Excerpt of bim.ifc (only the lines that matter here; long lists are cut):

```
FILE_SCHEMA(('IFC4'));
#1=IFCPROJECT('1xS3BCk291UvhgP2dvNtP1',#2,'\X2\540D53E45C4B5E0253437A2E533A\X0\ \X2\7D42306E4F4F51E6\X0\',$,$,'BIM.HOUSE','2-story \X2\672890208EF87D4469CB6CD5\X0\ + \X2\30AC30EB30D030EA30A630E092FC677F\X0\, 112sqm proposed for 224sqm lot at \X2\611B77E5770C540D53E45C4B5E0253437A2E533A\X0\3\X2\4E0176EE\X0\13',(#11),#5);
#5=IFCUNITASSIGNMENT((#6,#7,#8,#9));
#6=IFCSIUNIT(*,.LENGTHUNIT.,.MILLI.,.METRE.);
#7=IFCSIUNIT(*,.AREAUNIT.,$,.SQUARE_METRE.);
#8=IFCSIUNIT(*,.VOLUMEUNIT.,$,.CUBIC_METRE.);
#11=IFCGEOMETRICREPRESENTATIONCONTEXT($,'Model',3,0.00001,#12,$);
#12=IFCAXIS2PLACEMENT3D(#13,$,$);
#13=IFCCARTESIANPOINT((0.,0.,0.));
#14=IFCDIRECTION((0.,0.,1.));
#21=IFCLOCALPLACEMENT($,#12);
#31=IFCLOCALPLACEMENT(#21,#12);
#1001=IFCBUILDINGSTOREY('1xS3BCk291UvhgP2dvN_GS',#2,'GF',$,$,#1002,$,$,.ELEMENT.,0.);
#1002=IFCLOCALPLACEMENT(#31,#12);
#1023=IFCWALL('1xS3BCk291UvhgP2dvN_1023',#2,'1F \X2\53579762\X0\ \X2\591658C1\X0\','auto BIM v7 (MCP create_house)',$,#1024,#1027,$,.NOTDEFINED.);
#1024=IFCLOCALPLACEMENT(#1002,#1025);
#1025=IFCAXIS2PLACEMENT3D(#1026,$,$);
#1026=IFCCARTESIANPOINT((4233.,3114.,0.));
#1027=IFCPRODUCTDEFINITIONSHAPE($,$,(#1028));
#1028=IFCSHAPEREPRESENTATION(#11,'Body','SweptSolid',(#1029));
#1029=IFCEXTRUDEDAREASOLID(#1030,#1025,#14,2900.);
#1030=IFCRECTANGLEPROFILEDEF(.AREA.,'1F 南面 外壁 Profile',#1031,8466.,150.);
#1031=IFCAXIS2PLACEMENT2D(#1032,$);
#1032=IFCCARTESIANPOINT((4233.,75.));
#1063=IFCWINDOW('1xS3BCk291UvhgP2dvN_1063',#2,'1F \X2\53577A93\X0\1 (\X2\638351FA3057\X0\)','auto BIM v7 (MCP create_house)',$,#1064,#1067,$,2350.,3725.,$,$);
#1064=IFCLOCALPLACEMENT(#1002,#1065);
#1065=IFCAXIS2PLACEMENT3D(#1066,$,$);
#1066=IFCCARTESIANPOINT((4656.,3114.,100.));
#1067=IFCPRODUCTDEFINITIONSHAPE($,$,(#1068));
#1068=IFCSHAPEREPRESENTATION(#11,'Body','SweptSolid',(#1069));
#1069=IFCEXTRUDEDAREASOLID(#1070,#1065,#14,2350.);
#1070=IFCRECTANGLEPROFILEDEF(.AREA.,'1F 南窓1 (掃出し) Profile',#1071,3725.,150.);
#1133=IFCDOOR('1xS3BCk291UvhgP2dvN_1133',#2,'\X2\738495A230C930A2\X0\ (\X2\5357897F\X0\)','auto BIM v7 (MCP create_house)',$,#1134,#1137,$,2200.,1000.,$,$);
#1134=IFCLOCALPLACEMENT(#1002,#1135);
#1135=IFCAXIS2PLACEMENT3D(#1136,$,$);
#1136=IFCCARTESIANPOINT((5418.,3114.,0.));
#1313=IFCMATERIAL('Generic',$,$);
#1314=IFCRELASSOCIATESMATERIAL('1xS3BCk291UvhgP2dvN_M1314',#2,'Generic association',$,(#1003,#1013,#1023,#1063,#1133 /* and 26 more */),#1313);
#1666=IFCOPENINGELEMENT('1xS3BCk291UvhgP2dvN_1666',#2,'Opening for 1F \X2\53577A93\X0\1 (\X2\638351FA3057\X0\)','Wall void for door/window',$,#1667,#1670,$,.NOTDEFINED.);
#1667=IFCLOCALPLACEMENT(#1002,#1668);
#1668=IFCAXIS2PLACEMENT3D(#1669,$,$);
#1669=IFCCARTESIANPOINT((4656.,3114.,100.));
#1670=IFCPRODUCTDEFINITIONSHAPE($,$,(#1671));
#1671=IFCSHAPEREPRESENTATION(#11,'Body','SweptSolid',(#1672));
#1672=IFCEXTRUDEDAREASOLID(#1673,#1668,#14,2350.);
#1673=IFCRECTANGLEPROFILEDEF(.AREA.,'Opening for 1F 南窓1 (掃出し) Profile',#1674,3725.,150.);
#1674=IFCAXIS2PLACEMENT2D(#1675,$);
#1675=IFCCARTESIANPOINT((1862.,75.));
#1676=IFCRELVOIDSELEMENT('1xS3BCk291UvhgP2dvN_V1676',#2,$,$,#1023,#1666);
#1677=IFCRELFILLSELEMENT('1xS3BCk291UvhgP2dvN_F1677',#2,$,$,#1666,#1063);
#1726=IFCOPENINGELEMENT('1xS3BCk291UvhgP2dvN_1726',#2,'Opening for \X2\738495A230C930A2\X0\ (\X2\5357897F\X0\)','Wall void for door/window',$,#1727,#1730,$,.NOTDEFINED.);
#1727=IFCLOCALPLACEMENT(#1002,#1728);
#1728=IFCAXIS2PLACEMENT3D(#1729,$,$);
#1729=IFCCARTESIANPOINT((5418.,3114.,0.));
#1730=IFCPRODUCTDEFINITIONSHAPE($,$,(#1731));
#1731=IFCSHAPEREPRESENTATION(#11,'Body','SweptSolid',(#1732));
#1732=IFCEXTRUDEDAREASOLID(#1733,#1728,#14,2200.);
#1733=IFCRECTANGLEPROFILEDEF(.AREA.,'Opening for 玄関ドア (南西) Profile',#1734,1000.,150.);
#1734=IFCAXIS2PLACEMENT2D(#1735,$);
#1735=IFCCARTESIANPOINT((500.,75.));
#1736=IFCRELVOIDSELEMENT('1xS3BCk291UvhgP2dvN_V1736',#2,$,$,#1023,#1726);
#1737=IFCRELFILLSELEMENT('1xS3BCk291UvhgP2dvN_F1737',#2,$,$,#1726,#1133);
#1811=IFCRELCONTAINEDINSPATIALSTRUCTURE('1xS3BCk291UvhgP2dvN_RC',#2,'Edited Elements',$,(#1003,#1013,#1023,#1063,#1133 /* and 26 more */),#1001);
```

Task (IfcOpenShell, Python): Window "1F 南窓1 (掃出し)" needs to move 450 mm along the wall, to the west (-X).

```python
import ifcopenshell
import ifcopenshell.api.geometry
import ifcopenshell.util.placement
import ifcopenshell.util.unit

model = ifcopenshell.open("bim.ifc")
unit_scale = ifcopenshell.util.unit.calculate_unit_scale(model)

window = model.by_guid("1xS3BCk291UvhgP2dvN_1063")
opening = window.FillsVoids[0].RelatingOpeningElement
wall = opening.VoidsElements[0].RelatingBuildingElement

wall_matrix = ifcopenshell.util.placement.get_local_placement(wall.ObjectPlacement)
shift = wall_matrix[:3, 0] * -0.45 / unit_scale
before = ifcopenshell.util.placement.get_local_placement(window.ObjectPlacement)[:3, 3].copy()

# The window is not placed relative to its opening, so move both.
for product in (opening, window):
    matrix = ifcopenshell.util.placement.get_local_placement(product.ObjectPlacement)
    matrix[:3, 3] += shift
    ifcopenshell.api.geometry.edit_object_placement(model, product=product, matrix=matrix, is_si=False)

after = ifcopenshell.util.placement.get_local_placement(window.ObjectPlacement)[:3, 3]
print("window moved by", (after - before).round(3) + 0.0)

model.write("bim_rev.ifc")
```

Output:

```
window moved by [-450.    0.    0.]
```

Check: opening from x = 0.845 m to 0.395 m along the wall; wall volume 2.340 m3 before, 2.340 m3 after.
